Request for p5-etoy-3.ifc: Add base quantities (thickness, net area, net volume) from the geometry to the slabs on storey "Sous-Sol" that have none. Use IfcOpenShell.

First a look at what the model holds.

```python
import ifcopenshell
import ifcopenshell.util.element
import ifcopenshell.util.unit

model = ifcopenshell.open("p5-etoy-3.ifc")
print(model.schema)
for unit_type in ("LENGTHUNIT", "AREAUNIT", "VOLUMEUNIT"):
    print(unit_type, ifcopenshell.util.unit.calculate_unit_scale(model, unit_type))
storey = next(s for s in model.by_type("IfcBuildingStorey") if s.Name == "Sous-Sol")
slabs = [e for e in ifcopenshell.util.element.get_decomposition(storey) if e.is_a("IfcSlab")]
for e in sorted(slabs, key=lambda e: e.id()):
    print(e.id(), e.is_a(), e.Name, list(ifcopenshell.util.element.get_psets(e, qtos_only=True)), sep=" | ")
```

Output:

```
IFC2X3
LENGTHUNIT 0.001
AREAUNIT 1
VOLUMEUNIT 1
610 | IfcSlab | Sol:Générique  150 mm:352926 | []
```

```python
import ifcopenshell
import ifcopenshell.api.pset
import ifcopenshell.geom
import ifcopenshell.util.element
import ifcopenshell.util.shape
import ifcopenshell.util.unit

model = ifcopenshell.open("p5-etoy-3.ifc")
unit_scale = ifcopenshell.util.unit.calculate_unit_scale(model)
area_scale = ifcopenshell.util.unit.calculate_unit_scale(model, "AREAUNIT")
volume_scale = ifcopenshell.util.unit.calculate_unit_scale(model, "VOLUMEUNIT")
settings = ifcopenshell.geom.settings()

storey = next(s for s in model.by_type("IfcBuildingStorey") if s.Name == "Sous-Sol")
slabs = [e for e in ifcopenshell.util.element.get_decomposition(storey) if e.is_a("IfcSlab")]

for e in sorted(slabs, key=lambda e: e.id()):
    if ifcopenshell.util.element.get_psets(e, qtos_only=True, should_inherit=False):
        continue
    # Geometry comes back in metres, in the element's own axes.
    shape = ifcopenshell.geom.create_shape(settings, e)
    values = {
        "Width": ifcopenshell.util.shape.get_z(shape.geometry) / unit_scale,
        "NetArea": ifcopenshell.util.shape.get_footprint_area(shape.geometry) / area_scale,
        "NetVolume": ifcopenshell.util.shape.get_volume(shape.geometry) / volume_scale,
    }
    qto = ifcopenshell.api.pset.add_qto(model, product=e, name="BaseQuantities")
    ifcopenshell.api.pset.edit_qto(model, qto=qto, properties=values)
    print(e.id(), {k: round(v, 3) for k, v in values.items()})

model.write("p5-etoy-3_updated.ifc")
```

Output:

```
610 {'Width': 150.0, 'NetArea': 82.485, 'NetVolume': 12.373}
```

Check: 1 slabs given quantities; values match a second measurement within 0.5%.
